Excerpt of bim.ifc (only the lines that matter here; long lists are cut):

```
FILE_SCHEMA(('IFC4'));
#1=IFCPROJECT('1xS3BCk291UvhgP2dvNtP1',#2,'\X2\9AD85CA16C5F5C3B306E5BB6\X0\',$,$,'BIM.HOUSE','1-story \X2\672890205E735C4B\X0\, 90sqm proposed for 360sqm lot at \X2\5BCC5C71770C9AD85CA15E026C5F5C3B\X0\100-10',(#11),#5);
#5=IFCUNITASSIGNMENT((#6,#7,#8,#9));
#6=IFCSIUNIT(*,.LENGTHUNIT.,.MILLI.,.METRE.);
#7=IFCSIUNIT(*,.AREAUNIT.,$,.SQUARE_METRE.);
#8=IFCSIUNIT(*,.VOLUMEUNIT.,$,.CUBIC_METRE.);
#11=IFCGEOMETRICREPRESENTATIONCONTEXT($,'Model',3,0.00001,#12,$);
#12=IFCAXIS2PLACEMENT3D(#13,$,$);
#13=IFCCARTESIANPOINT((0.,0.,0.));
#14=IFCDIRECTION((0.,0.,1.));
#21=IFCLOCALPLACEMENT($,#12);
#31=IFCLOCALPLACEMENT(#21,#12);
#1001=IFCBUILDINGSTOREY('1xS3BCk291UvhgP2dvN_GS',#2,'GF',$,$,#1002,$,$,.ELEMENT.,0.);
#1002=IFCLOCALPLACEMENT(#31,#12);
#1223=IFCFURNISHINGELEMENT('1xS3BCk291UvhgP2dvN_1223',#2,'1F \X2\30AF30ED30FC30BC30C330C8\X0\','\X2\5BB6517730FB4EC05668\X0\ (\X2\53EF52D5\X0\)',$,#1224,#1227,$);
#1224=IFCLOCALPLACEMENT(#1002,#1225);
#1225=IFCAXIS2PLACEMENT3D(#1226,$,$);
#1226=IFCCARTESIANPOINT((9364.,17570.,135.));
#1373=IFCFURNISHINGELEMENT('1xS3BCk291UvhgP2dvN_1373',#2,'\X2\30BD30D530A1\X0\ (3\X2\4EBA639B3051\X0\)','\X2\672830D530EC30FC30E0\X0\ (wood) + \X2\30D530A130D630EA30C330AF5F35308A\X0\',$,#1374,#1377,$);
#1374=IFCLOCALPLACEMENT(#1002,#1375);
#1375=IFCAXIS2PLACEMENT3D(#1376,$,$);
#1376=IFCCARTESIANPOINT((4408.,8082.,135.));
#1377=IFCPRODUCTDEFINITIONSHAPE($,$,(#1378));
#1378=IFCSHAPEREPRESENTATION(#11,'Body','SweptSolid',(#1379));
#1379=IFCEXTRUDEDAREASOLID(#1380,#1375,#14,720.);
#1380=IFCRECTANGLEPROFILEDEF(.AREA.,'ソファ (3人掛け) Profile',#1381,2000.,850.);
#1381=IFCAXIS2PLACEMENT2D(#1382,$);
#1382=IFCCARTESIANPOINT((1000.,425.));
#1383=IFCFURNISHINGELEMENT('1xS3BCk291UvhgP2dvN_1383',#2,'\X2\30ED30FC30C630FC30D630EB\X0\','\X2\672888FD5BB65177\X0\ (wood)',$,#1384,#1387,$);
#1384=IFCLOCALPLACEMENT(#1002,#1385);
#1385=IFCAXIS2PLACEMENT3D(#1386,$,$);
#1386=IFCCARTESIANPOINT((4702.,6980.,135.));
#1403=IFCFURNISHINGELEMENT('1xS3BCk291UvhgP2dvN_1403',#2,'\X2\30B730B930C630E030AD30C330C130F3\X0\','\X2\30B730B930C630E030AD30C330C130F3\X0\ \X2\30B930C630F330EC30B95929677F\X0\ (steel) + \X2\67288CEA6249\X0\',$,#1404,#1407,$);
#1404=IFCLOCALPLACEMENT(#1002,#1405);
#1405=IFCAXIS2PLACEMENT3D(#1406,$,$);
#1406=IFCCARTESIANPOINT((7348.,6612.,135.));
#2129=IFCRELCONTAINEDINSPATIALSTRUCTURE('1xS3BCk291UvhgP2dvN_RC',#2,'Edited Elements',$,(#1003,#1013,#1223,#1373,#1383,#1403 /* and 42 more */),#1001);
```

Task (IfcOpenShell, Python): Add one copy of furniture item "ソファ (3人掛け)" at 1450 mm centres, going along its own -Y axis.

```python
import ifcopenshell
import ifcopenshell.api.geometry
import ifcopenshell.api.root
import ifcopenshell.util.element
import ifcopenshell.util.placement

model = ifcopenshell.open("bim.ifc")


def reuse_history(source, copy):
    """copy_class also copies each property set's owner history, people and application; keep the originals."""
    for rel in copy.IsDefinedBy:
        if rel.is_a("IfcRelDefinesByProperties") and (history := rel.RelatingPropertyDefinition.OwnerHistory):
            rel.RelatingPropertyDefinition.OwnerHistory = source.OwnerHistory
            ifcopenshell.util.element.remove_deep2(model, history)


source = model.by_guid("1xS3BCk291UvhgP2dvN_1373")
base = ifcopenshell.util.placement.get_local_placement(source.ObjectPlacement)
step = -base[:3, 1] * 1450.0

for i in range(1, 2):
    copy = ifcopenshell.api.root.copy_class(model, product=source)
    copy.Representation = ifcopenshell.util.element.copy_deep(
        model, source.Representation, exclude=["IfcGeometricRepresentationContext", "IfcRepresentationMap"]
    )
    reuse_history(source, copy)
    matrix = base.copy()
    matrix[:3, 3] += i * step
    print("added at", matrix[:3, 3].round(3) + 0.0)
    ifcopenshell.api.geometry.edit_object_placement(model, product=copy, matrix=matrix, is_si=False)

model.write("bim-out.ifc")
```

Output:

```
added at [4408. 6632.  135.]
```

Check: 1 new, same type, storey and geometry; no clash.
